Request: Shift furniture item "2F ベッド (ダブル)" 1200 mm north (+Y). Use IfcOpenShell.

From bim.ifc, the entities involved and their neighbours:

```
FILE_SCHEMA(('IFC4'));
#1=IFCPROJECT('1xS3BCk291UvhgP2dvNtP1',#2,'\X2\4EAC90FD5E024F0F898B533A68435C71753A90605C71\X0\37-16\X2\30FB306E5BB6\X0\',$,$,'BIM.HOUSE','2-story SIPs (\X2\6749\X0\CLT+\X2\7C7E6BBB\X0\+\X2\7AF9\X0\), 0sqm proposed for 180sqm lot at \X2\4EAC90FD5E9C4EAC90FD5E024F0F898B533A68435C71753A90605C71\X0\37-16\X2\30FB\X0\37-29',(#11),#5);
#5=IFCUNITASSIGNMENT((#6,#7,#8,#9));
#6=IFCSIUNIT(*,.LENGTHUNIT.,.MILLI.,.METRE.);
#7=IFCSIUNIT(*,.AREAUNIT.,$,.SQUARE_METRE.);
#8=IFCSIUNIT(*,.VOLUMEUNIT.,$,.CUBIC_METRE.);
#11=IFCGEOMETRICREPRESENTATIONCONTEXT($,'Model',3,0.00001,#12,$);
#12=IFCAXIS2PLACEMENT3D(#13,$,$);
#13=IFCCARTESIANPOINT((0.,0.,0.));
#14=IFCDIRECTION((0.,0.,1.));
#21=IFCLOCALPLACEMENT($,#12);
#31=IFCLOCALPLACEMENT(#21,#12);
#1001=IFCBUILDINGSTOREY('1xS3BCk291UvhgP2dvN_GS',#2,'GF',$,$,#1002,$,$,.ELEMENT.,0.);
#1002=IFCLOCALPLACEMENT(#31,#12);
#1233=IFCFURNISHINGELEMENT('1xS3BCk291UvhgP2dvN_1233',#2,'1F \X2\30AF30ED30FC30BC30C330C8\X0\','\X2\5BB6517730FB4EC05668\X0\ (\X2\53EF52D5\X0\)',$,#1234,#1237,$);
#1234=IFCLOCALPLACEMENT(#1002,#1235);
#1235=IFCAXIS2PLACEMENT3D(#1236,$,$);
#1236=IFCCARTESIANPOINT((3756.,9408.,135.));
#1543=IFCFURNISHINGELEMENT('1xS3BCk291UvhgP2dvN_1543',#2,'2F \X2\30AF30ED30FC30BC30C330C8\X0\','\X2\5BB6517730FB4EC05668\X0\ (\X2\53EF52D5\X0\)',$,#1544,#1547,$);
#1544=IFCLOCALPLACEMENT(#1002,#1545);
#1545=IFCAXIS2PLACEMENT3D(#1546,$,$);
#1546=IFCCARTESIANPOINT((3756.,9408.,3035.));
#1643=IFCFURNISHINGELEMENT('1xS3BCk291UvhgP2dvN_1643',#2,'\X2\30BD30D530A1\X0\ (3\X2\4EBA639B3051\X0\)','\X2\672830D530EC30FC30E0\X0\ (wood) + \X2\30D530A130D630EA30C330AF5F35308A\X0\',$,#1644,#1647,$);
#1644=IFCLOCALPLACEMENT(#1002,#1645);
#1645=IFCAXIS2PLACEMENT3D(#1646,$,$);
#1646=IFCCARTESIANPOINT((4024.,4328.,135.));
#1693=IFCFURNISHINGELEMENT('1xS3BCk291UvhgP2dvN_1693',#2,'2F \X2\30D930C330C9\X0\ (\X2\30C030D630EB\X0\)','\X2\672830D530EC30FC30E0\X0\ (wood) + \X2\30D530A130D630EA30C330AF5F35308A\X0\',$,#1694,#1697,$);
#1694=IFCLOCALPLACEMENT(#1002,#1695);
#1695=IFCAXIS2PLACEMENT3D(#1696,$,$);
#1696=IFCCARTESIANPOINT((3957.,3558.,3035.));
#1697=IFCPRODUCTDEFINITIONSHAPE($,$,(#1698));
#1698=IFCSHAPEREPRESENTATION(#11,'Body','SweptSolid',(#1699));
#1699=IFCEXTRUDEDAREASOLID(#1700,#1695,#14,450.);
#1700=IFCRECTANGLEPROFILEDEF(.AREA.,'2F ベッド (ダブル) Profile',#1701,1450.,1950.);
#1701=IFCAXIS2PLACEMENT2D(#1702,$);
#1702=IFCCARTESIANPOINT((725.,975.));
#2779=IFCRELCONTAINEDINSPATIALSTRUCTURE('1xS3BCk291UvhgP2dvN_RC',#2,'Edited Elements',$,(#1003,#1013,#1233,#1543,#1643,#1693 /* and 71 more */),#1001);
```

```python
import ifcopenshell
import ifcopenshell.api.geometry
import ifcopenshell.util.placement
import ifcopenshell.util.unit

model = ifcopenshell.open("bim.ifc")
unit_scale = ifcopenshell.util.unit.calculate_unit_scale(model)

item = model.by_guid("1xS3BCk291UvhgP2dvN_1693")
matrix = ifcopenshell.util.placement.get_local_placement(item.ObjectPlacement)
matrix[1, 3] += 1.2 / unit_scale
ifcopenshell.api.geometry.edit_object_placement(model, product=item, matrix=matrix, is_si=False)

print(ifcopenshell.util.placement.get_local_placement(item.ObjectPlacement).round(3) + 0.0)

model.write("bim_edited.ifc")
```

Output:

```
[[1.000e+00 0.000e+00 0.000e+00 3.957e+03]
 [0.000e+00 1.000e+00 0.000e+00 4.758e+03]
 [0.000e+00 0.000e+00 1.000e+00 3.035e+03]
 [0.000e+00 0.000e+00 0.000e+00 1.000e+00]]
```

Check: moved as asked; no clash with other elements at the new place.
